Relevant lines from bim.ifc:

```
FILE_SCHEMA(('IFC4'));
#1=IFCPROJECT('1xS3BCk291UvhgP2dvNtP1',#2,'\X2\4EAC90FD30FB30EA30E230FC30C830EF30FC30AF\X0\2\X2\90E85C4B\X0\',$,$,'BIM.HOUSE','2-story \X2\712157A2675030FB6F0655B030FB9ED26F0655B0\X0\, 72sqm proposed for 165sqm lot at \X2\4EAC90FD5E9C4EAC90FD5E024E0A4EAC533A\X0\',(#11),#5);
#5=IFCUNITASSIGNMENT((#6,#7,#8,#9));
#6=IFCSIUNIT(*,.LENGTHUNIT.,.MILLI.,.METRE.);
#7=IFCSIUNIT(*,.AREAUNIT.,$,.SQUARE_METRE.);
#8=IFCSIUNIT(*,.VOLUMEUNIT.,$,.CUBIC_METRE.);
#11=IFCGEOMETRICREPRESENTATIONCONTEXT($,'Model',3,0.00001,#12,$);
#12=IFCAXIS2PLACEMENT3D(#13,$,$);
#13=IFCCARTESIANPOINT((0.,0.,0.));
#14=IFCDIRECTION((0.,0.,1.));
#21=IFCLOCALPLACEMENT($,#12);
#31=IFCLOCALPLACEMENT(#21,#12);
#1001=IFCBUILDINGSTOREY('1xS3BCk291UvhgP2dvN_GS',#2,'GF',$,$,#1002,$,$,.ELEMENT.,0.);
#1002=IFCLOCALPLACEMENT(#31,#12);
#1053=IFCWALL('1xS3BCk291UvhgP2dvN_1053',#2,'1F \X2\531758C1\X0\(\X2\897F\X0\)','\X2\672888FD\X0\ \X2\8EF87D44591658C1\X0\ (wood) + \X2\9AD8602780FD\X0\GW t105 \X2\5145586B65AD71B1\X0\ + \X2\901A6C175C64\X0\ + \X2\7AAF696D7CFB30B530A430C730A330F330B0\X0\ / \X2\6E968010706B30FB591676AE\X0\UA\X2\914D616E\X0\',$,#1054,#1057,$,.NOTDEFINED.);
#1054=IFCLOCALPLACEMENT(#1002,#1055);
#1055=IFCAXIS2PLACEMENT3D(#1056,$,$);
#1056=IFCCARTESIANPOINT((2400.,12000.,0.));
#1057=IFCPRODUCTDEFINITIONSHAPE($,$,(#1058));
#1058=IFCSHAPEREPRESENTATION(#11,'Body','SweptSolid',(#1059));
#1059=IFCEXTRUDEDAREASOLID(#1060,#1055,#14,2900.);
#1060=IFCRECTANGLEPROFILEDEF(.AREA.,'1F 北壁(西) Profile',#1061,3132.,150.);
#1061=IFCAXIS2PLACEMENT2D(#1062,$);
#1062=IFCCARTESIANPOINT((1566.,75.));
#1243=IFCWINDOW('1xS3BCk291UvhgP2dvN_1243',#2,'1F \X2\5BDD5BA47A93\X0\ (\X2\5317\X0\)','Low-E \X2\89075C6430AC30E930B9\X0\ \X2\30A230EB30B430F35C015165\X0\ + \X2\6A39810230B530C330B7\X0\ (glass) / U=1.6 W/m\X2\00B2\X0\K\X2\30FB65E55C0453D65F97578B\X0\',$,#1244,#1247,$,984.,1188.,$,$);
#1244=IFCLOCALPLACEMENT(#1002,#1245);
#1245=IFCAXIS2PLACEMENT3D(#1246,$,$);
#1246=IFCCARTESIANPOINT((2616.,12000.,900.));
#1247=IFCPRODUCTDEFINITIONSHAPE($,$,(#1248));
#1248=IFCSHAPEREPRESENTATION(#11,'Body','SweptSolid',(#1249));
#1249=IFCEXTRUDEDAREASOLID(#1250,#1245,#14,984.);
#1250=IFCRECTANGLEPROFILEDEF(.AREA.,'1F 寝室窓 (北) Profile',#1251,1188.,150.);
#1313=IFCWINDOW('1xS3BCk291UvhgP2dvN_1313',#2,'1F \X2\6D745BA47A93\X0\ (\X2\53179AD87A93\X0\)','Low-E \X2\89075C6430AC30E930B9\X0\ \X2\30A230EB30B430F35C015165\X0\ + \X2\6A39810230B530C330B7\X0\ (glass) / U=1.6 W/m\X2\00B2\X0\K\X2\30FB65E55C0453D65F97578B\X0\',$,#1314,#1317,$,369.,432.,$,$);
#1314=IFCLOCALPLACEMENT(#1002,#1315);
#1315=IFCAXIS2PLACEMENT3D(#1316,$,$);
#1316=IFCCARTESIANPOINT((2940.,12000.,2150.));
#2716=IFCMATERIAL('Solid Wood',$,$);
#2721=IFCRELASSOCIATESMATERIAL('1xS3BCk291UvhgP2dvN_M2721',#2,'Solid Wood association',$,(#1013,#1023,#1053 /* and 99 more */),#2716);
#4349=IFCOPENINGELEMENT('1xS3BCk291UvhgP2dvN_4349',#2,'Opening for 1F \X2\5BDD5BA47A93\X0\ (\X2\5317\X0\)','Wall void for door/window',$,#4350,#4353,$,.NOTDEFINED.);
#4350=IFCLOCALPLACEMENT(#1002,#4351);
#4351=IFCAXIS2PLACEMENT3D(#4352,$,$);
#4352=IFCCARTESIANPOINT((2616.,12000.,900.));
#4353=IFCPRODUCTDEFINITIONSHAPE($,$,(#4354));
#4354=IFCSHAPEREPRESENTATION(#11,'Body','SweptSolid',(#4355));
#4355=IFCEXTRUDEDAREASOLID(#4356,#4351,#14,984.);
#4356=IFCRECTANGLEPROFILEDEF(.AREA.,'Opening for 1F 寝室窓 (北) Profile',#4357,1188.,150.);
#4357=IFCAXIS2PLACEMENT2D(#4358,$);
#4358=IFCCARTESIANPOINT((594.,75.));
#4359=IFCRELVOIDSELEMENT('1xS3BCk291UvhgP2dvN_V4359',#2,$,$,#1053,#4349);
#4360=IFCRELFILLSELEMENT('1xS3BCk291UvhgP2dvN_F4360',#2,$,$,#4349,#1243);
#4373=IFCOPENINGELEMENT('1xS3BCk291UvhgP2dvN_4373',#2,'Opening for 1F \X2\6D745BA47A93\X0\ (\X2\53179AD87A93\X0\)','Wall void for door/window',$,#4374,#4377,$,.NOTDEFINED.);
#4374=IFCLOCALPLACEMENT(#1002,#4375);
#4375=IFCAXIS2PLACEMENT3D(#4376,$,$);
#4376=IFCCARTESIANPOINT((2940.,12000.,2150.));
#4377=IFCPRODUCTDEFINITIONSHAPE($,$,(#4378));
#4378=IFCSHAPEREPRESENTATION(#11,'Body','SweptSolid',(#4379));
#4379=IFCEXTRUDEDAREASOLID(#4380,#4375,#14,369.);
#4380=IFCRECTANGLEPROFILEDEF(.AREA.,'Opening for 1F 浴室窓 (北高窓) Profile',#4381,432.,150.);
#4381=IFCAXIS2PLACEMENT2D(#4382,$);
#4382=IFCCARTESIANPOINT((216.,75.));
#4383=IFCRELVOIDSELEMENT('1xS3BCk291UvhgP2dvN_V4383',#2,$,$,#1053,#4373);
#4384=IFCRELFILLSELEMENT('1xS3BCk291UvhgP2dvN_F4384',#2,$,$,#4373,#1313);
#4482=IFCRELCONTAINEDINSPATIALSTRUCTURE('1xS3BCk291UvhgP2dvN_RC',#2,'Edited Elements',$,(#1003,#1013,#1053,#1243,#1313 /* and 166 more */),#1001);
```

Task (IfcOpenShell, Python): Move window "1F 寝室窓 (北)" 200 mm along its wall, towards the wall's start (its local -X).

```python
import ifcopenshell
import ifcopenshell.api.geometry
import ifcopenshell.util.placement

model = ifcopenshell.open("bim.ifc")

window = model.by_guid("1xS3BCk291UvhgP2dvN_1243")
opening = window.FillsVoids[0].RelatingOpeningElement
wall = opening.VoidsElements[0].RelatingBuildingElement

wall_matrix = ifcopenshell.util.placement.get_local_placement(wall.ObjectPlacement)
shift = wall_matrix[:3, 0] * -200.0
before = ifcopenshell.util.placement.get_local_placement(window.ObjectPlacement)[:3, 3].copy()

# The window is not placed relative to its opening, so move both.
for product in (opening, window):
    matrix = ifcopenshell.util.placement.get_local_placement(product.ObjectPlacement)
    matrix[:3, 3] += shift
    ifcopenshell.api.geometry.edit_object_placement(model, product=product, matrix=matrix, is_si=False)

after = ifcopenshell.util.placement.get_local_placement(window.ObjectPlacement)[:3, 3]
print("window moved by", (after - before).round(3) + 0.0)

model.write("bim_v2.ifc")
```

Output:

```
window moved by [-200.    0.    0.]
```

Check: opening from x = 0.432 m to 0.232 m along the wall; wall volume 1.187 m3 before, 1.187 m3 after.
